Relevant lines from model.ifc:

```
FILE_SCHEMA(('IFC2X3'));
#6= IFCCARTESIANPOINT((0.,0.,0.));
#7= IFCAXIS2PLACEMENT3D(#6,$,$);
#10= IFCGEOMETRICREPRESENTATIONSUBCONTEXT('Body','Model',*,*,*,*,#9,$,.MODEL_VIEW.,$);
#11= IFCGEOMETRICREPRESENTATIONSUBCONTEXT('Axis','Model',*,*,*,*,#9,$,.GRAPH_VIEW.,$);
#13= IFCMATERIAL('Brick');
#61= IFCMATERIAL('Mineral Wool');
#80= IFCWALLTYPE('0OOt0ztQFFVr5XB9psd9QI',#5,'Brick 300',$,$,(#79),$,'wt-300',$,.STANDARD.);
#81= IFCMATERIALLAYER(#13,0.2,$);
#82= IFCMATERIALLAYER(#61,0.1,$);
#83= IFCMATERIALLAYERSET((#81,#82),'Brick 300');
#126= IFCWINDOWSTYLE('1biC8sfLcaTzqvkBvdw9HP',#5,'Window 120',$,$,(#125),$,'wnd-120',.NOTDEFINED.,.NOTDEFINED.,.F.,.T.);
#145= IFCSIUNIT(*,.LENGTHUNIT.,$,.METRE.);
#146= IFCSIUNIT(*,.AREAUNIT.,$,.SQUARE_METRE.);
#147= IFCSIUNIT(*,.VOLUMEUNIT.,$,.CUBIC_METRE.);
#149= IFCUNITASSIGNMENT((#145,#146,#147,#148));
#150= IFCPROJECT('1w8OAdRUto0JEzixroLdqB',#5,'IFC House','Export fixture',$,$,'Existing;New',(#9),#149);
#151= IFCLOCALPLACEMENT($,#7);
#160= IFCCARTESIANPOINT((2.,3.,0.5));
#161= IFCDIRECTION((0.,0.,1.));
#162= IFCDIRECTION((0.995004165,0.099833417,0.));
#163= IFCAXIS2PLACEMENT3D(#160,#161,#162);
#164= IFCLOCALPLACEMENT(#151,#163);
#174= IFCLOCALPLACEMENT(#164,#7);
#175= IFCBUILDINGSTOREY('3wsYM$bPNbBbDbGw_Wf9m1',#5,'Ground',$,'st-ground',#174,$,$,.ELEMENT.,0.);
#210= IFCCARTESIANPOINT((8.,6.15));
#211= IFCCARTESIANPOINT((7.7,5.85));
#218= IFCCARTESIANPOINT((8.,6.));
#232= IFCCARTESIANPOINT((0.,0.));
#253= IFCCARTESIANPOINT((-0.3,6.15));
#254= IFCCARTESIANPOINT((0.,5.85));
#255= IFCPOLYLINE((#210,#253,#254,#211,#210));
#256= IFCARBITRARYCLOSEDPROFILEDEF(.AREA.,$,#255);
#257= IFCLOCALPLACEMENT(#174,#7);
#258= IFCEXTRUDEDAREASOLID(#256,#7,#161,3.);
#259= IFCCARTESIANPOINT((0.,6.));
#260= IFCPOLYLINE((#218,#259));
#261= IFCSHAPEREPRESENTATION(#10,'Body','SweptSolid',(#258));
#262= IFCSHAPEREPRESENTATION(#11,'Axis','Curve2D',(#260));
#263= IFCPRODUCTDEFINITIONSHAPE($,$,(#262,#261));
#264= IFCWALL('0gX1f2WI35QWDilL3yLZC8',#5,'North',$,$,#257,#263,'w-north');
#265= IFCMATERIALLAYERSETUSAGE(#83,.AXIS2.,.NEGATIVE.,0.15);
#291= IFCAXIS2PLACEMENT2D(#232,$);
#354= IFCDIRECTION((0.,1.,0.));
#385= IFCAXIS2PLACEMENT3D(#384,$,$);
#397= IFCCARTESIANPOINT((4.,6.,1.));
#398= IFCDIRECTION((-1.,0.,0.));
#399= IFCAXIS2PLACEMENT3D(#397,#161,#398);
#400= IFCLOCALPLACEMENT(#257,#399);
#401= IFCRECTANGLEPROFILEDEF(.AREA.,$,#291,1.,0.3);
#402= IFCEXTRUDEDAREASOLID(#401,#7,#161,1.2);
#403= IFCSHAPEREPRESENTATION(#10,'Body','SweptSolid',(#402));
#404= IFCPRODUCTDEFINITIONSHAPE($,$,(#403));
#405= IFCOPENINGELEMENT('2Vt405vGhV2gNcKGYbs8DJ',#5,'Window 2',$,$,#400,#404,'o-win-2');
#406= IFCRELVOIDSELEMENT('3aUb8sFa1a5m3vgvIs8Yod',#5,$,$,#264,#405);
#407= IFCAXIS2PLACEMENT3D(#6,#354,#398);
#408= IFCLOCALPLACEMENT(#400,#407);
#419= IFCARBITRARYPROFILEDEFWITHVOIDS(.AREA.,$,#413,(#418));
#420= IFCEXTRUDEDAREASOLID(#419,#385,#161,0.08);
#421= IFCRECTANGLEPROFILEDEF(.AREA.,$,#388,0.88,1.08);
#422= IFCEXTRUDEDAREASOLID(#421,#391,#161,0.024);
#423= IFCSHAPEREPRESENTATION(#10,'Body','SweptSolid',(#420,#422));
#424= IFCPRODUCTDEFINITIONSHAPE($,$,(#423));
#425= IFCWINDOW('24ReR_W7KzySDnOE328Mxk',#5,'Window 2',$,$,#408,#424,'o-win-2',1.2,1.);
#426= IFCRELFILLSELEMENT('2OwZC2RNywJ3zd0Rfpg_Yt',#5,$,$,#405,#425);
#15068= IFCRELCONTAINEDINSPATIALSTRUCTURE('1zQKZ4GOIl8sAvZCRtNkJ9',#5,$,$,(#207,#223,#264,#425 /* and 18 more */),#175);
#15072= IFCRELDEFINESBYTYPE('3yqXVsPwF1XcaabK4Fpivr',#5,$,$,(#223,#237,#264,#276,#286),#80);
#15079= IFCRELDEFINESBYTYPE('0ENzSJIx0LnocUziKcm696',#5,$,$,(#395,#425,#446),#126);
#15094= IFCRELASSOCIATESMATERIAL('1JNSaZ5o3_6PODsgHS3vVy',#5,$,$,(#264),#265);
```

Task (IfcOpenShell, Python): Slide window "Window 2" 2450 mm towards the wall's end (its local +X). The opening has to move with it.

```python
import ifcopenshell
import ifcopenshell.api.geometry
import ifcopenshell.util.placement

model = ifcopenshell.open("model.ifc")

window = model.by_guid("24ReR_W7KzySDnOE328Mxk")
opening = window.FillsVoids[0].RelatingOpeningElement
wall = opening.VoidsElements[0].RelatingBuildingElement

wall_matrix = ifcopenshell.util.placement.get_local_placement(wall.ObjectPlacement)
shift = wall_matrix[:3, 0] * 2.45
before = ifcopenshell.util.placement.get_local_placement(window.ObjectPlacement)[:3, 3].copy()

# The window is placed relative to its opening, so it follows when the opening moves.
matrix = ifcopenshell.util.placement.get_local_placement(opening.ObjectPlacement)
matrix[:3, 3] += shift
ifcopenshell.api.geometry.edit_object_placement(
    model, product=opening, matrix=matrix, is_si=False, should_transform_children=True
)

after = ifcopenshell.util.placement.get_local_placement(window.ObjectPlacement)[:3, 3]
print("window moved by", (after - before).round(3) + 0.0)

model.write("model_rev.ifc")
```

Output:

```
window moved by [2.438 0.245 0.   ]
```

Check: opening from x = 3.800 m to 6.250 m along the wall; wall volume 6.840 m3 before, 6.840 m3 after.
